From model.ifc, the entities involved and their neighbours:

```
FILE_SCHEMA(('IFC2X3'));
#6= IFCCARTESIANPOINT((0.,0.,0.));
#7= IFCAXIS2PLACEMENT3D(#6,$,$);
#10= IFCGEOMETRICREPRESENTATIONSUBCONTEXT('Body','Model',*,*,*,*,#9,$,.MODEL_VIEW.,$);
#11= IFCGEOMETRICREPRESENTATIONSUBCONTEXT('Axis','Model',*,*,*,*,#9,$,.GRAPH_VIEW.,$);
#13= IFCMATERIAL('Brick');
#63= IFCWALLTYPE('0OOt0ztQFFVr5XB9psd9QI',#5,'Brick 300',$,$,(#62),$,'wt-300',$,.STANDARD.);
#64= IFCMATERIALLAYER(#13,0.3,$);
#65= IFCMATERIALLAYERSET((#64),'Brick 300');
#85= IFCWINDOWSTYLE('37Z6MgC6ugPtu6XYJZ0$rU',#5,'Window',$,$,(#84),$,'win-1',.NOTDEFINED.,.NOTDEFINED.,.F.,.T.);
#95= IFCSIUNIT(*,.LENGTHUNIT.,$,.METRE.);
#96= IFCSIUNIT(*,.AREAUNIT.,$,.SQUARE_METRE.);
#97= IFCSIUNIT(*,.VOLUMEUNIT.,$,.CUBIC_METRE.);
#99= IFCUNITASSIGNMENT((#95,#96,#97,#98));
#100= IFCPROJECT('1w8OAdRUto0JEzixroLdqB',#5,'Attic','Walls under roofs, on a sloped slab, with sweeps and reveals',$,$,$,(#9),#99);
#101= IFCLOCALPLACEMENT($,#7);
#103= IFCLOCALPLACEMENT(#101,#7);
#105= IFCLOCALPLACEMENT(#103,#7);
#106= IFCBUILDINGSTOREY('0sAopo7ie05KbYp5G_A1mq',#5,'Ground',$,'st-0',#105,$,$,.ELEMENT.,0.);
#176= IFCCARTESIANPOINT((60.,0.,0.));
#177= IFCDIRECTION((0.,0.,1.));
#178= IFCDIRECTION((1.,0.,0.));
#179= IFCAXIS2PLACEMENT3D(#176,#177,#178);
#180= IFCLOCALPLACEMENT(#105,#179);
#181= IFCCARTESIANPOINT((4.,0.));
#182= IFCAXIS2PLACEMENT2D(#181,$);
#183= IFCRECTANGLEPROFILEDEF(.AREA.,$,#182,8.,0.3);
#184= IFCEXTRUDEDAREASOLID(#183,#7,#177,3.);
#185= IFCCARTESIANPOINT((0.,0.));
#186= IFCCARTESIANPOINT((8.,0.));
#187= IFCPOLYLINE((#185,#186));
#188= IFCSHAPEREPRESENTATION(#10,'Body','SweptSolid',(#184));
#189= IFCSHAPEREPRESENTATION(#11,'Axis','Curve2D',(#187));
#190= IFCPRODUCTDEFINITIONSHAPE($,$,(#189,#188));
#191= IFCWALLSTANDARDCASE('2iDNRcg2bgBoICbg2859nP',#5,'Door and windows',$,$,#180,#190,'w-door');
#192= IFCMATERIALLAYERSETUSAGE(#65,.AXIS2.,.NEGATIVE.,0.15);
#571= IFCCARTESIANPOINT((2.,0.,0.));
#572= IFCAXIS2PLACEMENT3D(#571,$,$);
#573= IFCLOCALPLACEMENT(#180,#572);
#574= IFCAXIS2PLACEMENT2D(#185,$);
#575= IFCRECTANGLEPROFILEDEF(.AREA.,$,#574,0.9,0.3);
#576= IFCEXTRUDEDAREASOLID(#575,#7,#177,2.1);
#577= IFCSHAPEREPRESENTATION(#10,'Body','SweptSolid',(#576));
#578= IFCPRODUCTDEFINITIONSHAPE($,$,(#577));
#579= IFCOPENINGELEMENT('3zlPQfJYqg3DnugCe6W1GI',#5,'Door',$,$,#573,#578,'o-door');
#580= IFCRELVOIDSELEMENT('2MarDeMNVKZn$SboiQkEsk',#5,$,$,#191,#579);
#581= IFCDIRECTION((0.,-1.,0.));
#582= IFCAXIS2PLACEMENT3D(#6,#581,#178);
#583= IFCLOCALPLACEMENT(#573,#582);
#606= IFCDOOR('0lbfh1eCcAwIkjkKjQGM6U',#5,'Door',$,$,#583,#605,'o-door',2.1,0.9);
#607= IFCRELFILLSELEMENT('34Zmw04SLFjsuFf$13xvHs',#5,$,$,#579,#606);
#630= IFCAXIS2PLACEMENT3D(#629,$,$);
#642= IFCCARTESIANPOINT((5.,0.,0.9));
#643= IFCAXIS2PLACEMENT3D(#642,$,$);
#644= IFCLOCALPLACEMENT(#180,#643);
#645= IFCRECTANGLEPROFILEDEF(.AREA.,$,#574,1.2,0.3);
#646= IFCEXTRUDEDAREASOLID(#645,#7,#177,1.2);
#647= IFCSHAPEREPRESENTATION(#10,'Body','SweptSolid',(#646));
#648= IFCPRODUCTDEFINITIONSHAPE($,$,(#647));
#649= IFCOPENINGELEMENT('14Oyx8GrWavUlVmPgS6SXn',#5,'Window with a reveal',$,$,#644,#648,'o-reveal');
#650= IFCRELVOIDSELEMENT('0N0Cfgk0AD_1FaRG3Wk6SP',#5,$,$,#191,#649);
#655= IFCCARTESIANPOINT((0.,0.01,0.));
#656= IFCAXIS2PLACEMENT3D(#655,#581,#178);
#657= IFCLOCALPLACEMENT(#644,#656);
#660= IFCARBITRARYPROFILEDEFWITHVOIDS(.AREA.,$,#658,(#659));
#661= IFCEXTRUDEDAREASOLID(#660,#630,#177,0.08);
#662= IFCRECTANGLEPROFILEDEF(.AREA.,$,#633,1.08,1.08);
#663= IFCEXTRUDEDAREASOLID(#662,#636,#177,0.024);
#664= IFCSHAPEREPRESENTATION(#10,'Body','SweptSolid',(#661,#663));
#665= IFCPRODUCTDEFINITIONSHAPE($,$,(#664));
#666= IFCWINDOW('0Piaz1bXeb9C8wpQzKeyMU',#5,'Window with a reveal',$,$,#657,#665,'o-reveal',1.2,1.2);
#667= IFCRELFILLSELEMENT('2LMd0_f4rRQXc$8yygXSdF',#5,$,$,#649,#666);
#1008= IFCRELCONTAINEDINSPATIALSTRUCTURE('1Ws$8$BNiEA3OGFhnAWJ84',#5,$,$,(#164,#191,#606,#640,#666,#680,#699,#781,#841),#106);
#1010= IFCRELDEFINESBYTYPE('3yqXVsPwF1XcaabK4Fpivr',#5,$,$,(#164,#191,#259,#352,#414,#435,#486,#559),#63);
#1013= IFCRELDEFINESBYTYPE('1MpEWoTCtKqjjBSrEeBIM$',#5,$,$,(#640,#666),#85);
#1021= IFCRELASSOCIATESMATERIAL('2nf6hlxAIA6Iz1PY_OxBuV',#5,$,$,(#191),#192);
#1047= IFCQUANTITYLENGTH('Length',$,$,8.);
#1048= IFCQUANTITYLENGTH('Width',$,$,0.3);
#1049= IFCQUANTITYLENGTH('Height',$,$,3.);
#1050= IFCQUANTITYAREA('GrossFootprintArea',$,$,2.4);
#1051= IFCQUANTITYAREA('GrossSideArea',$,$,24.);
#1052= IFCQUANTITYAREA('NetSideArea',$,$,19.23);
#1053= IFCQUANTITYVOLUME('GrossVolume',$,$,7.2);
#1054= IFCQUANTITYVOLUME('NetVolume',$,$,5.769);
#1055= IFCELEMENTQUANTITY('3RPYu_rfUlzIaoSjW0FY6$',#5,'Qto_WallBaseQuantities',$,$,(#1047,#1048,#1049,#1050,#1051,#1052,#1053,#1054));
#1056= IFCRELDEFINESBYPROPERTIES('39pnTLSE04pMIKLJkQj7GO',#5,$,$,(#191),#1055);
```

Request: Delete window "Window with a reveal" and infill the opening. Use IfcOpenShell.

```python
import ifcopenshell
import ifcopenshell.api.feature
import ifcopenshell.api.pset
import ifcopenshell.api.root
import ifcopenshell.geom
import ifcopenshell.util.element
import ifcopenshell.util.shape
import ifcopenshell.util.unit

model = ifcopenshell.open("model.ifc")
area_scale = ifcopenshell.util.unit.calculate_unit_scale(model, "AREAUNIT")
volume_scale = ifcopenshell.util.unit.calculate_unit_scale(model, "VOLUMEUNIT")
settings = ifcopenshell.geom.settings()


def volume(element):
    """Net volume in cubic metres, openings subtracted."""
    shape = ifcopenshell.geom.create_shape(settings, element)
    return ifcopenshell.util.shape.get_volume(shape.geometry)


window = model.by_id(666)
opening = window.FillsVoids[0].RelatingOpeningElement
wall = opening.VoidsElements[0].RelatingBuildingElement
before = volume(wall)

ifcopenshell.api.root.remove_product(model, product=window)
ifcopenshell.api.feature.remove_feature(model, feature=opening)

after = volume(wall)
thickness = 0.3  # wall thickness in metres

# Update the wall's stored quantities.
qto = model.by_id(ifcopenshell.util.element.get_pset(wall, "Qto_WallBaseQuantities", should_inherit=False)["id"])
ifcopenshell.api.pset.edit_qto(model, qto=qto, properties={
    "NetSideArea": after / thickness / area_scale,
    "NetVolume": after / volume_scale,
})

print(f"wall volume {before:.3f} -> {after:.3f} m3")

model.write("model_updated.ifc")
```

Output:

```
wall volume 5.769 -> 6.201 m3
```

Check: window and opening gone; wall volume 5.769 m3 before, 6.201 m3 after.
